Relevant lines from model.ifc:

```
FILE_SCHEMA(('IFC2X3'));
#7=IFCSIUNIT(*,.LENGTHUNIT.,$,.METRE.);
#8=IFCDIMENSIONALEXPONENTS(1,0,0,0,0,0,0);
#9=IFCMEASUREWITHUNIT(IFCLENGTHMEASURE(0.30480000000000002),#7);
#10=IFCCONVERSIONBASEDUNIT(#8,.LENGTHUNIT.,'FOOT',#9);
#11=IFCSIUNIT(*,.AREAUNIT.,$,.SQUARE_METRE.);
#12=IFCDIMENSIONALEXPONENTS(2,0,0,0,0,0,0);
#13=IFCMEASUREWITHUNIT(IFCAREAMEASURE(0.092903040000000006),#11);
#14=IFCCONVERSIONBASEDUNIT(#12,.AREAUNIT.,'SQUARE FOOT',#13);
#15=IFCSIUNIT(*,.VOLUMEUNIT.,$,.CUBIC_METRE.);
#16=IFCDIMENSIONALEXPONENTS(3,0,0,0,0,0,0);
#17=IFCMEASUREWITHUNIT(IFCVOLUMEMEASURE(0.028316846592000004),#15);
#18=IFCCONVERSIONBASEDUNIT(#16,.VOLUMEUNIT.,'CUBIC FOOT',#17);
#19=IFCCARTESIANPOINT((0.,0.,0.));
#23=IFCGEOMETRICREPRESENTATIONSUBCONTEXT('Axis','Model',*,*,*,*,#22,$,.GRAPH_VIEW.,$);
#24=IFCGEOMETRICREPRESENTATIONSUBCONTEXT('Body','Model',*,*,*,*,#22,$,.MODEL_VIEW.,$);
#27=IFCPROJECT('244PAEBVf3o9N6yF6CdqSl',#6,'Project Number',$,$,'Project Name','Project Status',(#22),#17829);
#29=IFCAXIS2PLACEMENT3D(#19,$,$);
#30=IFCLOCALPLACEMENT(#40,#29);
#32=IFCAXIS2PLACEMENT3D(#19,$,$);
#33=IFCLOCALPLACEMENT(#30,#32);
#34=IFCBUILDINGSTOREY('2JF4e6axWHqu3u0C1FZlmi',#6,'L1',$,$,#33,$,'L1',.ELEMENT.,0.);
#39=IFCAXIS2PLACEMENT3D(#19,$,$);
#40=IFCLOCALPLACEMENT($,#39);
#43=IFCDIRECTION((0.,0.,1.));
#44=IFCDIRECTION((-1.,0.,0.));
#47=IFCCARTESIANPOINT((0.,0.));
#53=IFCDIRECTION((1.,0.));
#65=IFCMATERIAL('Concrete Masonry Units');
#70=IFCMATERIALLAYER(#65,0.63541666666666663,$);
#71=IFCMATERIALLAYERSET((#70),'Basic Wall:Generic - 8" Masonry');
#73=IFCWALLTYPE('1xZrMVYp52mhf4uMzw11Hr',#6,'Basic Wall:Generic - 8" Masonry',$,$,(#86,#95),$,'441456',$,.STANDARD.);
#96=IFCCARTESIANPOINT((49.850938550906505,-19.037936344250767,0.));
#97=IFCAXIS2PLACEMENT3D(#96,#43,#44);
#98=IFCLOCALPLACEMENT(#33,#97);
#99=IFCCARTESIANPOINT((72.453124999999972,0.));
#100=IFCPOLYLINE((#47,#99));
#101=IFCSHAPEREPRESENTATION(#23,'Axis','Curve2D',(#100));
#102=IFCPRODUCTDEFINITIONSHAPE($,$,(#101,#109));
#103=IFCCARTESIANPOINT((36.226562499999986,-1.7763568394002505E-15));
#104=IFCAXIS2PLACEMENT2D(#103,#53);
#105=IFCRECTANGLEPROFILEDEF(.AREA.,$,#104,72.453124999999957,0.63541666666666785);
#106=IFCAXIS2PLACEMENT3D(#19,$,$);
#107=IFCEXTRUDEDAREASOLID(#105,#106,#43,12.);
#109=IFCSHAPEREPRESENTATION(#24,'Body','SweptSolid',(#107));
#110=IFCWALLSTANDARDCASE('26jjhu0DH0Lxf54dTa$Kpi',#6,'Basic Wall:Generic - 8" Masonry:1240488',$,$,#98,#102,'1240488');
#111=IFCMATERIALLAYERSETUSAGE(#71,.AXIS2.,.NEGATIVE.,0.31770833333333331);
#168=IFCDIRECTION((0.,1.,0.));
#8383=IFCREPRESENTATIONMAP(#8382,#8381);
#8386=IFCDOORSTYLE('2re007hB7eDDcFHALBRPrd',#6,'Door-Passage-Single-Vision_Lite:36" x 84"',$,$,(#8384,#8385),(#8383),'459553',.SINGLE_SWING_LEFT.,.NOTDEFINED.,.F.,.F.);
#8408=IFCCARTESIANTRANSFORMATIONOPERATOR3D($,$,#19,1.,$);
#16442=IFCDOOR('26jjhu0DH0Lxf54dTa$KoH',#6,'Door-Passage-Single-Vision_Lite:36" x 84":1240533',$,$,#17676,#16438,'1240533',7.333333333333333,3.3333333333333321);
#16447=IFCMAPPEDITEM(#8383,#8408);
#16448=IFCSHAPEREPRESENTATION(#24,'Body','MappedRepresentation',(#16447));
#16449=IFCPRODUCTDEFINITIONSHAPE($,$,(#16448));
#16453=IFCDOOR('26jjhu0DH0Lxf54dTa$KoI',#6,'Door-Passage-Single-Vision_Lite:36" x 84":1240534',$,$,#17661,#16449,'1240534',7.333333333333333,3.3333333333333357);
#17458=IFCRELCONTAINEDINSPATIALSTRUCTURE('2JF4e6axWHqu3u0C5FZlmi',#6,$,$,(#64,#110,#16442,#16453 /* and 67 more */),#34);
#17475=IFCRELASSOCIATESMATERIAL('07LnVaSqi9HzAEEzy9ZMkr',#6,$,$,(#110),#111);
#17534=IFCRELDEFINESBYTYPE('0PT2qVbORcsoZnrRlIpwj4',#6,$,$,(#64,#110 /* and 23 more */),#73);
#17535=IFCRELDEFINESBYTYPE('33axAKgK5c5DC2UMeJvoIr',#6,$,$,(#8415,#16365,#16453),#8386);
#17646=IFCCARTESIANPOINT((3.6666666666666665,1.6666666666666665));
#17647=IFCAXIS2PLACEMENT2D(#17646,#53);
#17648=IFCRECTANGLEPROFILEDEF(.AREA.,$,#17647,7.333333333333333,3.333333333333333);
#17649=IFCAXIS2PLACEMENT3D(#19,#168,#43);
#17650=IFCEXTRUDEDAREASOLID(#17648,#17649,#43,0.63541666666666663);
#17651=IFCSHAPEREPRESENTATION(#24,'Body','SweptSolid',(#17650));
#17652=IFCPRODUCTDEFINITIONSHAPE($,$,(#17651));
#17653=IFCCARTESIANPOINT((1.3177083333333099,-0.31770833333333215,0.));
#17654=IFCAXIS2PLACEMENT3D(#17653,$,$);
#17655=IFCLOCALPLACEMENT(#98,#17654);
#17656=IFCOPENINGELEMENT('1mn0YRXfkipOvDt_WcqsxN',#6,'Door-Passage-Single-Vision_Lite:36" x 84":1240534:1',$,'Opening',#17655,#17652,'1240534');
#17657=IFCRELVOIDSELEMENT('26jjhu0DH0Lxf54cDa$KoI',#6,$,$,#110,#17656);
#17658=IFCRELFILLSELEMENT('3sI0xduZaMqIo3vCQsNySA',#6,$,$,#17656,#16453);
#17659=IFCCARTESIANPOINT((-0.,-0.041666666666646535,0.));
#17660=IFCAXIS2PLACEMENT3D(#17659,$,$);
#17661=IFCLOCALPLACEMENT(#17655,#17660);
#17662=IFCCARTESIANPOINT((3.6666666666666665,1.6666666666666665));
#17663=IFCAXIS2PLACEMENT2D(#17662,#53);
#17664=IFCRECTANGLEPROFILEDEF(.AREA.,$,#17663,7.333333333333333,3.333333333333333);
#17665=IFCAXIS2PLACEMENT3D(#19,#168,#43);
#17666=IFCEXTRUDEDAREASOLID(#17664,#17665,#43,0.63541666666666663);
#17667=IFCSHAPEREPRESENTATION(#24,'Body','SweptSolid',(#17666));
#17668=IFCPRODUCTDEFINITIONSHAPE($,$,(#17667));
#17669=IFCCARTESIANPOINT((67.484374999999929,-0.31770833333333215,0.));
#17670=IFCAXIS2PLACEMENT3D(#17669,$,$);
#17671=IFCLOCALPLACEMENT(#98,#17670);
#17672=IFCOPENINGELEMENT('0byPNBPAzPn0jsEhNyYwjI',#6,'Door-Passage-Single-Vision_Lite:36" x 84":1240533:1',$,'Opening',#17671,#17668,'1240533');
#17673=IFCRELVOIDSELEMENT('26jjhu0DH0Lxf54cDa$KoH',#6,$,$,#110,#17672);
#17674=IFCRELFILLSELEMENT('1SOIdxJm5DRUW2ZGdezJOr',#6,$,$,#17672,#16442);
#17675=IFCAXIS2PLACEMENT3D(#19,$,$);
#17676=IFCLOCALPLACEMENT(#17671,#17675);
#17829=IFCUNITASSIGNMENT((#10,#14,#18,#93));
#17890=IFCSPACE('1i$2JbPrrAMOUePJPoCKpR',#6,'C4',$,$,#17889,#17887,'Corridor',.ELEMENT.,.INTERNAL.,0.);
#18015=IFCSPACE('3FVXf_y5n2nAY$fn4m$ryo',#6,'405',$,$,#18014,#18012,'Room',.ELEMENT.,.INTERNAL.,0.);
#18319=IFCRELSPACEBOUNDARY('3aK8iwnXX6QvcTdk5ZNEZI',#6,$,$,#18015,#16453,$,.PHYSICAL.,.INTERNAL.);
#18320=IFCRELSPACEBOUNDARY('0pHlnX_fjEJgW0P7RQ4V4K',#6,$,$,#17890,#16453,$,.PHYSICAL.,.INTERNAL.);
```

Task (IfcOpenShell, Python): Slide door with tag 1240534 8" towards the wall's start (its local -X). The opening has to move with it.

```python
import ifcopenshell
import ifcopenshell.api.geometry
import ifcopenshell.util.placement
import ifcopenshell.util.unit

model = ifcopenshell.open("model.ifc")
unit_scale = ifcopenshell.util.unit.calculate_unit_scale(model)

door = model.by_id(16453)
opening = door.FillsVoids[0].RelatingOpeningElement
wall = opening.VoidsElements[0].RelatingBuildingElement

wall_matrix = ifcopenshell.util.placement.get_local_placement(wall.ObjectPlacement)
shift = wall_matrix[:3, 0] * -8 * 0.0254 / unit_scale
before = ifcopenshell.util.placement.get_local_placement(door.ObjectPlacement)[:3, 3].copy()

# The door is placed relative to its opening, so it follows when the opening moves.
matrix = ifcopenshell.util.placement.get_local_placement(opening.ObjectPlacement)
matrix[:3, 3] += shift
ifcopenshell.api.geometry.edit_object_placement(
    model, product=opening, matrix=matrix, is_si=False, should_transform_children=True
)

after = ifcopenshell.util.placement.get_local_placement(door.ObjectPlacement)[:3, 3]
print("door moved by", (after - before).round(3) + 0.0)

model.write("model_updated.ifc")
```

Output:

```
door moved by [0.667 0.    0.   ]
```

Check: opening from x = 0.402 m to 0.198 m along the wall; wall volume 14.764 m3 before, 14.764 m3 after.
